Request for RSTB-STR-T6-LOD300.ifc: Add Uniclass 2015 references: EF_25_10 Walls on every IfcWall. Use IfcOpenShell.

First a look at what the model holds.

```python
import ifcopenshell

model = ifcopenshell.open("RSTB-STR-T6-LOD300.ifc")
print(model.schema)
print("classifications:", [c.Name for c in model.by_type("IfcClassification")])
for ifc_class in ("IfcDoor", "IfcRoof", "IfcStair", "IfcWall", "IfcWindow"):
    print(ifc_class, len(model.by_type(ifc_class)))
```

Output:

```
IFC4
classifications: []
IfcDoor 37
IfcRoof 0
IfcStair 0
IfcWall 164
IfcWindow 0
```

```python
import ifcopenshell
import ifcopenshell.api.classification

model = ifcopenshell.open("RSTB-STR-T6-LOD300.ifc")

system = ifcopenshell.api.classification.add_classification(model, classification="Uniclass 2015")

codes = {
    "IfcWall": ("EF_25_10", "Walls"),
}
for ifc_class, (code, name) in codes.items():
    products = model.by_type(ifc_class)
    ifcopenshell.api.classification.add_reference(
        model, products=products, classification=system, identification=code, name=name
    )
    print(code, len(products))

model.write("RSTB-STR-T6-LOD300_v2.ifc")
```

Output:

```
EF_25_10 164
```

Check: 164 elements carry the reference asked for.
